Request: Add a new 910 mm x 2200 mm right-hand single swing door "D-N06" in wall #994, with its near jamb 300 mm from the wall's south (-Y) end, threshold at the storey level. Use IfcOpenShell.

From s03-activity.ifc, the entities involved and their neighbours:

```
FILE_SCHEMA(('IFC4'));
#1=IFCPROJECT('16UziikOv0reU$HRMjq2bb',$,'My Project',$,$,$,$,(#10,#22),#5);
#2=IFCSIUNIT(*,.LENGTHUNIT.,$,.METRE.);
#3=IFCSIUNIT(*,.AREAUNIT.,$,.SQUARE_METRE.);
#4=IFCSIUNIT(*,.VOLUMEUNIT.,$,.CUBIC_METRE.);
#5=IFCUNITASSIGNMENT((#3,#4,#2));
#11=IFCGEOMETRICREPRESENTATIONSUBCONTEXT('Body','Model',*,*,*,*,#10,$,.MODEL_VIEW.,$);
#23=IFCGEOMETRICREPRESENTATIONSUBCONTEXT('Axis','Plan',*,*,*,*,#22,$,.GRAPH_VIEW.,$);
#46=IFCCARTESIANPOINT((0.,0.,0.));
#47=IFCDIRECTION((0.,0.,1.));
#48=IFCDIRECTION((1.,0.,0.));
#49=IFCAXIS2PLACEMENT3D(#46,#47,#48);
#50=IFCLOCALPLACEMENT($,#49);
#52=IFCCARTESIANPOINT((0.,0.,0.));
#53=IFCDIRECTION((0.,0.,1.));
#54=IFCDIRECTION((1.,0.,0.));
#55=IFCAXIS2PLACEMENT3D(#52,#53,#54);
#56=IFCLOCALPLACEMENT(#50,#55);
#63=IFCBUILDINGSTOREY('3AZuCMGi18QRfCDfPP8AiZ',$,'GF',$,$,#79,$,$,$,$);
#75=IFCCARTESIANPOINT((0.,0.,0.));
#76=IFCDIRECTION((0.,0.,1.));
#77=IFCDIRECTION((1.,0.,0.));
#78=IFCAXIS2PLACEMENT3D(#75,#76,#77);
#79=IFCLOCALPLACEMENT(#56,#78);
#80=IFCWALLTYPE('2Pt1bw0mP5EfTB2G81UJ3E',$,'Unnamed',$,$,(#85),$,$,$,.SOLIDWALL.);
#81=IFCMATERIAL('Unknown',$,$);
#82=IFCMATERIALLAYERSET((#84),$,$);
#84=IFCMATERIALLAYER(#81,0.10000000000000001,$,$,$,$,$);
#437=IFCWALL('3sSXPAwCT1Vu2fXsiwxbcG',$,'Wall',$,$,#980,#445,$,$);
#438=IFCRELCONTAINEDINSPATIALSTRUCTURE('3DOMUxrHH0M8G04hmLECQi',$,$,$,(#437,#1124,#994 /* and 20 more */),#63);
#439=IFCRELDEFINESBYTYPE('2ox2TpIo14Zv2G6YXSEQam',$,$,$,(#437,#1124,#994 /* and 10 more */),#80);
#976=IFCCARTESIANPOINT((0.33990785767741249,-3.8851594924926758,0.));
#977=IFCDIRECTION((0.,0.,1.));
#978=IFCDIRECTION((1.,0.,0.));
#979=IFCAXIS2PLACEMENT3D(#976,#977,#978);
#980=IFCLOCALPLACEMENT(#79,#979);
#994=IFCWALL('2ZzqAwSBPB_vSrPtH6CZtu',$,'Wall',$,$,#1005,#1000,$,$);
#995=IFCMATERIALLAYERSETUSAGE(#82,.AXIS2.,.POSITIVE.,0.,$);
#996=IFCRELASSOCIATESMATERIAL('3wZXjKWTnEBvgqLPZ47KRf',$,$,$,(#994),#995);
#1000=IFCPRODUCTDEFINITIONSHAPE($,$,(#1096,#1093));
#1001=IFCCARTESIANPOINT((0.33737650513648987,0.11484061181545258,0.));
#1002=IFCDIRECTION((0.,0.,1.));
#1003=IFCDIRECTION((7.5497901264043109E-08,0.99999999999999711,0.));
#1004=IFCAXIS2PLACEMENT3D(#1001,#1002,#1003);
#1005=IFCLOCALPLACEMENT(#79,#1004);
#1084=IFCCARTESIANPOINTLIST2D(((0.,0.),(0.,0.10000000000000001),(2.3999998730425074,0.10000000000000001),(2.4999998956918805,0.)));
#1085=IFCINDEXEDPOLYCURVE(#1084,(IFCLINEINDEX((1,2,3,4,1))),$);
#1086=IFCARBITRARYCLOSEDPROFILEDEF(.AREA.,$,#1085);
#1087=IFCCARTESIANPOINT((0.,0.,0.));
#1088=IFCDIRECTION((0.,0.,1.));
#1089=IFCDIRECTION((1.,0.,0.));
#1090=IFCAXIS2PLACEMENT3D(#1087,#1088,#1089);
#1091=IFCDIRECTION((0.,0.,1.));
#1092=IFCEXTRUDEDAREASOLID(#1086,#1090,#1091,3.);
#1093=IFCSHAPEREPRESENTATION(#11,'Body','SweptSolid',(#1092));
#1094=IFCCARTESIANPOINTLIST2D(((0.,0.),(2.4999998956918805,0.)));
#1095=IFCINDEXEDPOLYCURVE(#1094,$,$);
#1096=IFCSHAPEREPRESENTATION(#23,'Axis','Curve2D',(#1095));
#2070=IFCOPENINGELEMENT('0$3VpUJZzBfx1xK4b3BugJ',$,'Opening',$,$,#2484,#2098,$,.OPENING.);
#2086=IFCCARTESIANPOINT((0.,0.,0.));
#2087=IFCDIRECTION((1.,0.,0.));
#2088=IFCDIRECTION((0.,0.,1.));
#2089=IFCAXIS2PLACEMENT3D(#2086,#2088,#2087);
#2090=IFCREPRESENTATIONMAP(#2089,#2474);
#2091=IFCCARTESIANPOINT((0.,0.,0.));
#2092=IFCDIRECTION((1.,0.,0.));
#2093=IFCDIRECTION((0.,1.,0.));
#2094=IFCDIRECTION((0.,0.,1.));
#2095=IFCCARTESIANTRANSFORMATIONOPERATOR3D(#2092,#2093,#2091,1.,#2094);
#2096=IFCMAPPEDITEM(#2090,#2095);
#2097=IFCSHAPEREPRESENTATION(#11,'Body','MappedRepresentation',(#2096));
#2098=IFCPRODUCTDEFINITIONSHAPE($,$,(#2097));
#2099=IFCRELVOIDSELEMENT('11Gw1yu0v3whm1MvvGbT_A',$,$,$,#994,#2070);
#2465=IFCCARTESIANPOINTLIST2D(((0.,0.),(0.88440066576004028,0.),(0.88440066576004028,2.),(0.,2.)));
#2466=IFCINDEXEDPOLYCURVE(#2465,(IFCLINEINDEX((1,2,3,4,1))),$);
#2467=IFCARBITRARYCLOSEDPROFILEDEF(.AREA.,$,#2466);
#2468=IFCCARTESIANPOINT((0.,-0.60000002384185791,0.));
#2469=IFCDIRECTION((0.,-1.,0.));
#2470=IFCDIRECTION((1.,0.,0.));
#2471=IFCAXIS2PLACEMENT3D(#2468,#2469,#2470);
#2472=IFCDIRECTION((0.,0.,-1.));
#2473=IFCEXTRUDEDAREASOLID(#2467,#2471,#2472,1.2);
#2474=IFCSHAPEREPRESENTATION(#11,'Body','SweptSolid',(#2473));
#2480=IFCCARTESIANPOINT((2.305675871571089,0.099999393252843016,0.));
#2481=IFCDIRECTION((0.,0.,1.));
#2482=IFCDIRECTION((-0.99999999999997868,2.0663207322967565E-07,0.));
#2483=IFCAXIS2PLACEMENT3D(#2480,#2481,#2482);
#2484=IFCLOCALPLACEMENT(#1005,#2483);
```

```python
import numpy as np
import ifcopenshell
import ifcopenshell.api.feature
import ifcopenshell.api.geometry
import ifcopenshell.api.root
import ifcopenshell.api.spatial
import ifcopenshell.geom
import ifcopenshell.util.element
import ifcopenshell.util.placement
import ifcopenshell.util.representation
import ifcopenshell.util.shape
import ifcopenshell.util.unit

model = ifcopenshell.open("s03-activity.ifc")
unit_scale = ifcopenshell.util.unit.calculate_unit_scale(model)
settings = ifcopenshell.geom.settings()


def volume(element):
    """Net volume in cubic metres, openings subtracted."""
    shape = ifcopenshell.geom.create_shape(settings, element)
    return ifcopenshell.util.shape.get_volume(shape.geometry)


wall = model.by_guid("2ZzqAwSBPB_vSrPtH6CZtu")
storey = ifcopenshell.util.element.get_container(wall, ifc_class="IfcBuildingStorey")
context = ifcopenshell.util.representation.get_context(model, "Model", "Body", "MODEL_VIEW")
before = volume(wall)

width, height, from_end, sill = 0.91, 2.2, 0.3, 0.0  # metres

# The wall runs along its own X axis, and the end named is its -X end.
wall_shape = ifcopenshell.geom.create_shape(settings, wall)
x, y, z = ifcopenshell.util.shape.get_vertices(wall_shape.geometry).T
start = x.min() + from_end
face, thickness = float(y.min()), float(y.max() - y.min())
wall_matrix = ifcopenshell.util.placement.get_local_placement(wall.ObjectPlacement)
level = ifcopenshell.util.placement.get_local_placement(storey.ObjectPlacement)[2, 3]


def in_wall(x, y):
    """Placement at x, y metres in the wall's axes, at sill height."""
    matrix = wall_matrix.copy()
    matrix[:, 3] = wall_matrix @ np.array([x / unit_scale, y / unit_scale, 0.0, 1.0])
    matrix[2, 3] = level + sill / unit_scale
    return matrix


# Opening: a box that overshoots both wall faces by 50 mm.
opening = ifcopenshell.api.root.create_entity(model, ifc_class="IfcOpeningElement", predefined_type="OPENING")
box = ifcopenshell.api.geometry.add_wall_representation(
    model, context=context, length=width, height=height, thickness=thickness + 0.1
)
ifcopenshell.api.geometry.assign_representation(model, product=opening, representation=box)
ifcopenshell.api.geometry.edit_object_placement(model, product=opening, matrix=in_wall(start, face - 0.05), is_si=False)
ifcopenshell.api.feature.add_feature(model, feature=opening, element=wall)

door = ifcopenshell.api.root.create_entity(model, ifc_class="IfcDoor", name="D-N06", predefined_type="DOOR")
door.OverallWidth, door.OverallHeight = width / unit_scale, height / unit_scale
door.OperationType = "SINGLE_SWING_RIGHT"
body = ifcopenshell.api.geometry.add_door_representation(
    model,
    context=context,
    overall_width=door.OverallWidth,
    overall_height=door.OverallHeight,
    operation_type="SINGLE_SWING_RIGHT",
    lining_properties={"LiningDepth": thickness / unit_scale, "ThresholdDepth": thickness / unit_scale},
)
ifcopenshell.api.geometry.assign_representation(model, product=door, representation=body)
ifcopenshell.api.spatial.assign_container(model, products=[door], relating_structure=storey)
ifcopenshell.api.feature.add_filling(model, opening=opening, element=door)

# The lining spans the wall, so the door starts at the wall face.
ifcopenshell.api.geometry.edit_object_placement(model, product=door, matrix=in_wall(start, face), is_si=False)

after = volume(wall)

print(f"wall volume {before:.3f} -> {after:.3f} m3")

model.write("s03-activity-out.ifc")
```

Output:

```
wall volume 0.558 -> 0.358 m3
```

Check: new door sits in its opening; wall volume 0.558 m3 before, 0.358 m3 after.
